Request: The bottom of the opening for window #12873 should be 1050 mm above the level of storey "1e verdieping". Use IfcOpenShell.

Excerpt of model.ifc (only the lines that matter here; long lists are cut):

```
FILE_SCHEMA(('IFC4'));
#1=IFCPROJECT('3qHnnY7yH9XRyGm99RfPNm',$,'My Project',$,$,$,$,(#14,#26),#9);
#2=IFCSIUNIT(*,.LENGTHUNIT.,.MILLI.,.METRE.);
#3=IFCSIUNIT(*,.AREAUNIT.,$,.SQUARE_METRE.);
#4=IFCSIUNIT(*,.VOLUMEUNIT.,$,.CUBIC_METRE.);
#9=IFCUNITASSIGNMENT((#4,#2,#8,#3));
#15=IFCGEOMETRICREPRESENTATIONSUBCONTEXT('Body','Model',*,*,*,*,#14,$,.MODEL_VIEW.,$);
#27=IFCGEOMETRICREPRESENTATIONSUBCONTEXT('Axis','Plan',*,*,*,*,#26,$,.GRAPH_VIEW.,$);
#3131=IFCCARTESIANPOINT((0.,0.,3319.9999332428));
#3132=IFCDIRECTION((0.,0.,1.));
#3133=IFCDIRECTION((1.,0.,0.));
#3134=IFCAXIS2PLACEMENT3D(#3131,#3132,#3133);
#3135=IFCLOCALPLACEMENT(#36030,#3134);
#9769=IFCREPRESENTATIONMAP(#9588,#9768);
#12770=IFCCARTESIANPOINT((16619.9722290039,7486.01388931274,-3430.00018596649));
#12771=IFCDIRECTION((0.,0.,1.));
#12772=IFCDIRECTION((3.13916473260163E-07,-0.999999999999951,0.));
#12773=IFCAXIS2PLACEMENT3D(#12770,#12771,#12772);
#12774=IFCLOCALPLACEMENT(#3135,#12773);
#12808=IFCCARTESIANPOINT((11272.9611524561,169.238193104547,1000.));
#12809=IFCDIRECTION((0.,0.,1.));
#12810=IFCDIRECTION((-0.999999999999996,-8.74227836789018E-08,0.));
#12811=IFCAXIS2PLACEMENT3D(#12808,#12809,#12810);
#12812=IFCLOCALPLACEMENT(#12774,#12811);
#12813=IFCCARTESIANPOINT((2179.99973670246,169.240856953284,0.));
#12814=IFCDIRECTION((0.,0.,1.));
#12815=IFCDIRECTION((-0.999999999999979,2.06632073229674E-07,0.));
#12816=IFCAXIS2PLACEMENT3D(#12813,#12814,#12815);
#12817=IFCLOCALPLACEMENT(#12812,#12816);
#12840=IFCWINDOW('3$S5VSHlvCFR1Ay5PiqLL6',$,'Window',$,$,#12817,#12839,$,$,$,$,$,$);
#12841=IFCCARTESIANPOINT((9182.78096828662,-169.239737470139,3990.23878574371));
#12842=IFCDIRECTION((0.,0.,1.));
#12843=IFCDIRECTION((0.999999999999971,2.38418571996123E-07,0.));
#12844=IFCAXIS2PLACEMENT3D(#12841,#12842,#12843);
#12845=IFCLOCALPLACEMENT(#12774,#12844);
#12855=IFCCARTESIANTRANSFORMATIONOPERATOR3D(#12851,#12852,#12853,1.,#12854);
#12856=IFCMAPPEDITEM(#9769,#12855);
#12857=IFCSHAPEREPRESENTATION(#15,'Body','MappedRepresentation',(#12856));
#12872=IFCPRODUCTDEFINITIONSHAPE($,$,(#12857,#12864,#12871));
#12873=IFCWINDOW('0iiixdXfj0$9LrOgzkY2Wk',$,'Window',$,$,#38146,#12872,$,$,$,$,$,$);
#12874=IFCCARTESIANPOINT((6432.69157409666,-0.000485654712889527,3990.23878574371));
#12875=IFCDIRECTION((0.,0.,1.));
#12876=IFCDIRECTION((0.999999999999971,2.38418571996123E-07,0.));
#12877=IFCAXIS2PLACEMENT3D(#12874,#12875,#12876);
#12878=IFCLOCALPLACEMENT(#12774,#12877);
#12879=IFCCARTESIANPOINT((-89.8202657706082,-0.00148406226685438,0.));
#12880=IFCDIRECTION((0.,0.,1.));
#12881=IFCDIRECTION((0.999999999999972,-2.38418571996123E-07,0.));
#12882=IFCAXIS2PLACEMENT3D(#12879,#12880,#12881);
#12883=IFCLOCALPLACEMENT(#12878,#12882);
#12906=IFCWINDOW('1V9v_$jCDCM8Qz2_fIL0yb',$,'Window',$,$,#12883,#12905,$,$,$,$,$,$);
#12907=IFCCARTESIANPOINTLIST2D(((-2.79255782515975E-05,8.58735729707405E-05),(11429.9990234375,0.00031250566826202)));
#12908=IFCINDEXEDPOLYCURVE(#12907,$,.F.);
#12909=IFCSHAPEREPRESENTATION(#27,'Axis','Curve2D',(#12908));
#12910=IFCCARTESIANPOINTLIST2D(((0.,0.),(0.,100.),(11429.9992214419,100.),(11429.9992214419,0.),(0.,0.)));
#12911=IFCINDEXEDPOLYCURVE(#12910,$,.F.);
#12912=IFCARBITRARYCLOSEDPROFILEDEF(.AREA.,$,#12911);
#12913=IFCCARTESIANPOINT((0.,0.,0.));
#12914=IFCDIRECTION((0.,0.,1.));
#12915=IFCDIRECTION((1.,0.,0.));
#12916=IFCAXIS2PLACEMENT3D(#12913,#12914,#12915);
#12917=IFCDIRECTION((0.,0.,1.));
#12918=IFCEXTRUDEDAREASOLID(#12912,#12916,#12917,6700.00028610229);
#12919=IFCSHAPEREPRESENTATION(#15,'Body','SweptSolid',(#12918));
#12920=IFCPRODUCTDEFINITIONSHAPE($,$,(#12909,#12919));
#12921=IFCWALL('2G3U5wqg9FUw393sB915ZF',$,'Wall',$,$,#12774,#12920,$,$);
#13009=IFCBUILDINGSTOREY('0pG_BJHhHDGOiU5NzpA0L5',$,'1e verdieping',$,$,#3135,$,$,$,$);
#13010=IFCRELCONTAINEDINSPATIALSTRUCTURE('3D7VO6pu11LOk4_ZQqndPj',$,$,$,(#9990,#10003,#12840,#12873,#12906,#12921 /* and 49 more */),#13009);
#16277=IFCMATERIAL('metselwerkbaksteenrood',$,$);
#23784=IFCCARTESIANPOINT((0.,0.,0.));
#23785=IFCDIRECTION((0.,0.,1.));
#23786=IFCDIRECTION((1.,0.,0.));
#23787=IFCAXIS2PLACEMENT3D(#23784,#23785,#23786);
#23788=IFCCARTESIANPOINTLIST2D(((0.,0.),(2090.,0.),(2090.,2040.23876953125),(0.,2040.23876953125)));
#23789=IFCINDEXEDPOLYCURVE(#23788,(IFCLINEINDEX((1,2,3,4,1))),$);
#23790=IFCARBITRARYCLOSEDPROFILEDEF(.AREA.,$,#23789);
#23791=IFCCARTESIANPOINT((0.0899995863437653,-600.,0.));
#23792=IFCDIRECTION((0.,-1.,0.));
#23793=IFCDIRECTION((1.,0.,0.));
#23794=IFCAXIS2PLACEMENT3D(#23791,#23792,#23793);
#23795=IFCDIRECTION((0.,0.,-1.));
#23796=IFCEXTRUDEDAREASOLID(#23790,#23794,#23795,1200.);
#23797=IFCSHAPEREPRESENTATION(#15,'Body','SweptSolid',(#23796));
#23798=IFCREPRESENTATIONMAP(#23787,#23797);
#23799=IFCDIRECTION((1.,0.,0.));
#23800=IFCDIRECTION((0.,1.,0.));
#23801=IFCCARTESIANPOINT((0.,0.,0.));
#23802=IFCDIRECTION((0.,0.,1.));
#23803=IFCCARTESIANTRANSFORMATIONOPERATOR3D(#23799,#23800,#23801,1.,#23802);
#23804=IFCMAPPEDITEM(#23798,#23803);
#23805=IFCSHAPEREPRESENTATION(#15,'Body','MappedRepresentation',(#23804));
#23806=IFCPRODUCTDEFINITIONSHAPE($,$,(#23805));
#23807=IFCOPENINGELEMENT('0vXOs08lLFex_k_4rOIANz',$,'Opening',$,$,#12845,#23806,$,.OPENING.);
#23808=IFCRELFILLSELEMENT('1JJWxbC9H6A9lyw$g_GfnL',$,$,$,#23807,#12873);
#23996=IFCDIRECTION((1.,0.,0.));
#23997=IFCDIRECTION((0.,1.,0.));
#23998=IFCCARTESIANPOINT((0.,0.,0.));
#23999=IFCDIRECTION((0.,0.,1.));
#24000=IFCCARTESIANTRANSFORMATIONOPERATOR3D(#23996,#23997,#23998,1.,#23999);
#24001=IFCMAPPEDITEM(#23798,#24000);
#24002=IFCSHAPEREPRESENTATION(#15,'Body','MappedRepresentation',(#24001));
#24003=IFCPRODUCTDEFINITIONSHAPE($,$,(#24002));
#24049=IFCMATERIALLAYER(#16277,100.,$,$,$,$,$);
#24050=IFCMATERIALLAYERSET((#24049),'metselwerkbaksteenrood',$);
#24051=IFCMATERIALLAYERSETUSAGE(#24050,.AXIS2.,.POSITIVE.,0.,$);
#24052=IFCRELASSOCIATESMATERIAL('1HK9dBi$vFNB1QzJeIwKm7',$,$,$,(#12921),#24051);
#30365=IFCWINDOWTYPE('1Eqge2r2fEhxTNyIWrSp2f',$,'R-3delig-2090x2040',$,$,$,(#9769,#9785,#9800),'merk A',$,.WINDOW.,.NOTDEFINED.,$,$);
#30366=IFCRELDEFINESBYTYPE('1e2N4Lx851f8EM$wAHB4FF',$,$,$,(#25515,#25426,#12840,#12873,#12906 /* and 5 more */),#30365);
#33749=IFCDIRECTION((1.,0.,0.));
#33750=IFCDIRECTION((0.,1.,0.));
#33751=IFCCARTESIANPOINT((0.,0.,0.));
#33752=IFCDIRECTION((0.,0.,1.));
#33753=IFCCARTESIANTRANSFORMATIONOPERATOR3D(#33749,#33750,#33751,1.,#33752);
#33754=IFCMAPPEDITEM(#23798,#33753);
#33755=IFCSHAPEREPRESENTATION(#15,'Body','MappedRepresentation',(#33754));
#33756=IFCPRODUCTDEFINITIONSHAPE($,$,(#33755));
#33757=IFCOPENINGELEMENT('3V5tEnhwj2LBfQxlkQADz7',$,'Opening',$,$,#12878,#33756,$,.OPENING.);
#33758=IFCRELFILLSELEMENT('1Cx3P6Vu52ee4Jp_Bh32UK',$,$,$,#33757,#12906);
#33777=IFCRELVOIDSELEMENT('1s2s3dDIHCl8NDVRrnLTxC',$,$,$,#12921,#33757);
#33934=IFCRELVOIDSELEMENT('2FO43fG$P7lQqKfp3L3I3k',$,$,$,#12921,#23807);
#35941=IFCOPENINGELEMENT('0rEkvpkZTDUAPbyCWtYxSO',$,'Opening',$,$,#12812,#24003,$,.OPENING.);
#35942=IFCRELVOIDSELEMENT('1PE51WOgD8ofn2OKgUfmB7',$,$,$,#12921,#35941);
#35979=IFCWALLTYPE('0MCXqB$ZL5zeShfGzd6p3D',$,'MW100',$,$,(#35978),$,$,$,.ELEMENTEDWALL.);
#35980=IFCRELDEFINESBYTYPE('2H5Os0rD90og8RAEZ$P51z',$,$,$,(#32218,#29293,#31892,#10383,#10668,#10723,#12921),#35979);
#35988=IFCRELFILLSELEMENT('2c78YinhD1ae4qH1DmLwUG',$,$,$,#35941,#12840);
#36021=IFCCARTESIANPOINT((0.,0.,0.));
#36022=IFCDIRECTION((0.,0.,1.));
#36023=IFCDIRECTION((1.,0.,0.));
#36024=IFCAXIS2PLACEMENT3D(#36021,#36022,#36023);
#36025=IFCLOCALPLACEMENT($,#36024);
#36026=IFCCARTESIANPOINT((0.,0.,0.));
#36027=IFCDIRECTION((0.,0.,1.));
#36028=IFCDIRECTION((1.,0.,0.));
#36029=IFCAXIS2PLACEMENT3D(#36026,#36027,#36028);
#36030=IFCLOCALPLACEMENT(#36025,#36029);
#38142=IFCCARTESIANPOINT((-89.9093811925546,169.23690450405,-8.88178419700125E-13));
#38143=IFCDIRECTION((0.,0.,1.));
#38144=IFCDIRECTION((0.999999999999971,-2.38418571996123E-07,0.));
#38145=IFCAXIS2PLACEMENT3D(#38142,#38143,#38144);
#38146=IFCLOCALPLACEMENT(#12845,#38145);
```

```python
import numpy as np
import ifcopenshell
import ifcopenshell.api.geometry
import ifcopenshell.geom
import ifcopenshell.util.element
import ifcopenshell.util.placement
import ifcopenshell.util.shape
import ifcopenshell.util.unit

model = ifcopenshell.open("model.ifc")
unit_scale = ifcopenshell.util.unit.calculate_unit_scale(model)

window = model.by_guid("0iiixdXfj0$9LrOgzkY2Wk")
opening = window.FillsVoids[0].RelatingOpeningElement
storey = ifcopenshell.util.element.get_container(window, ifc_class="IfcBuildingStorey")
level = ifcopenshell.util.placement.get_local_placement(storey.ObjectPlacement)[2, 3]

# The opening's origin need not be at the sill, so measure its lowest point.
shape = ifcopenshell.geom.create_shape(ifcopenshell.geom.settings(), opening)
bottom = ifcopenshell.util.shape.get_shape_bottom_elevation(shape, shape.geometry) / unit_scale
dz = level + 1050.0 - bottom

shift = np.array([0.0, 0.0, dz])
# The window is placed relative to its opening, so it follows when the opening moves.
matrix = ifcopenshell.util.placement.get_local_placement(opening.ObjectPlacement)
matrix[:3, 3] += shift
ifcopenshell.api.geometry.edit_object_placement(
    model, product=opening, matrix=matrix, is_si=False, should_transform_children=True
)

print(f"moved by {dz * unit_scale:+.3f} m")

model.write("model_updated.ifc")
```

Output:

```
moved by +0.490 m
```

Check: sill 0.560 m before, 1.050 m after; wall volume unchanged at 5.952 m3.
